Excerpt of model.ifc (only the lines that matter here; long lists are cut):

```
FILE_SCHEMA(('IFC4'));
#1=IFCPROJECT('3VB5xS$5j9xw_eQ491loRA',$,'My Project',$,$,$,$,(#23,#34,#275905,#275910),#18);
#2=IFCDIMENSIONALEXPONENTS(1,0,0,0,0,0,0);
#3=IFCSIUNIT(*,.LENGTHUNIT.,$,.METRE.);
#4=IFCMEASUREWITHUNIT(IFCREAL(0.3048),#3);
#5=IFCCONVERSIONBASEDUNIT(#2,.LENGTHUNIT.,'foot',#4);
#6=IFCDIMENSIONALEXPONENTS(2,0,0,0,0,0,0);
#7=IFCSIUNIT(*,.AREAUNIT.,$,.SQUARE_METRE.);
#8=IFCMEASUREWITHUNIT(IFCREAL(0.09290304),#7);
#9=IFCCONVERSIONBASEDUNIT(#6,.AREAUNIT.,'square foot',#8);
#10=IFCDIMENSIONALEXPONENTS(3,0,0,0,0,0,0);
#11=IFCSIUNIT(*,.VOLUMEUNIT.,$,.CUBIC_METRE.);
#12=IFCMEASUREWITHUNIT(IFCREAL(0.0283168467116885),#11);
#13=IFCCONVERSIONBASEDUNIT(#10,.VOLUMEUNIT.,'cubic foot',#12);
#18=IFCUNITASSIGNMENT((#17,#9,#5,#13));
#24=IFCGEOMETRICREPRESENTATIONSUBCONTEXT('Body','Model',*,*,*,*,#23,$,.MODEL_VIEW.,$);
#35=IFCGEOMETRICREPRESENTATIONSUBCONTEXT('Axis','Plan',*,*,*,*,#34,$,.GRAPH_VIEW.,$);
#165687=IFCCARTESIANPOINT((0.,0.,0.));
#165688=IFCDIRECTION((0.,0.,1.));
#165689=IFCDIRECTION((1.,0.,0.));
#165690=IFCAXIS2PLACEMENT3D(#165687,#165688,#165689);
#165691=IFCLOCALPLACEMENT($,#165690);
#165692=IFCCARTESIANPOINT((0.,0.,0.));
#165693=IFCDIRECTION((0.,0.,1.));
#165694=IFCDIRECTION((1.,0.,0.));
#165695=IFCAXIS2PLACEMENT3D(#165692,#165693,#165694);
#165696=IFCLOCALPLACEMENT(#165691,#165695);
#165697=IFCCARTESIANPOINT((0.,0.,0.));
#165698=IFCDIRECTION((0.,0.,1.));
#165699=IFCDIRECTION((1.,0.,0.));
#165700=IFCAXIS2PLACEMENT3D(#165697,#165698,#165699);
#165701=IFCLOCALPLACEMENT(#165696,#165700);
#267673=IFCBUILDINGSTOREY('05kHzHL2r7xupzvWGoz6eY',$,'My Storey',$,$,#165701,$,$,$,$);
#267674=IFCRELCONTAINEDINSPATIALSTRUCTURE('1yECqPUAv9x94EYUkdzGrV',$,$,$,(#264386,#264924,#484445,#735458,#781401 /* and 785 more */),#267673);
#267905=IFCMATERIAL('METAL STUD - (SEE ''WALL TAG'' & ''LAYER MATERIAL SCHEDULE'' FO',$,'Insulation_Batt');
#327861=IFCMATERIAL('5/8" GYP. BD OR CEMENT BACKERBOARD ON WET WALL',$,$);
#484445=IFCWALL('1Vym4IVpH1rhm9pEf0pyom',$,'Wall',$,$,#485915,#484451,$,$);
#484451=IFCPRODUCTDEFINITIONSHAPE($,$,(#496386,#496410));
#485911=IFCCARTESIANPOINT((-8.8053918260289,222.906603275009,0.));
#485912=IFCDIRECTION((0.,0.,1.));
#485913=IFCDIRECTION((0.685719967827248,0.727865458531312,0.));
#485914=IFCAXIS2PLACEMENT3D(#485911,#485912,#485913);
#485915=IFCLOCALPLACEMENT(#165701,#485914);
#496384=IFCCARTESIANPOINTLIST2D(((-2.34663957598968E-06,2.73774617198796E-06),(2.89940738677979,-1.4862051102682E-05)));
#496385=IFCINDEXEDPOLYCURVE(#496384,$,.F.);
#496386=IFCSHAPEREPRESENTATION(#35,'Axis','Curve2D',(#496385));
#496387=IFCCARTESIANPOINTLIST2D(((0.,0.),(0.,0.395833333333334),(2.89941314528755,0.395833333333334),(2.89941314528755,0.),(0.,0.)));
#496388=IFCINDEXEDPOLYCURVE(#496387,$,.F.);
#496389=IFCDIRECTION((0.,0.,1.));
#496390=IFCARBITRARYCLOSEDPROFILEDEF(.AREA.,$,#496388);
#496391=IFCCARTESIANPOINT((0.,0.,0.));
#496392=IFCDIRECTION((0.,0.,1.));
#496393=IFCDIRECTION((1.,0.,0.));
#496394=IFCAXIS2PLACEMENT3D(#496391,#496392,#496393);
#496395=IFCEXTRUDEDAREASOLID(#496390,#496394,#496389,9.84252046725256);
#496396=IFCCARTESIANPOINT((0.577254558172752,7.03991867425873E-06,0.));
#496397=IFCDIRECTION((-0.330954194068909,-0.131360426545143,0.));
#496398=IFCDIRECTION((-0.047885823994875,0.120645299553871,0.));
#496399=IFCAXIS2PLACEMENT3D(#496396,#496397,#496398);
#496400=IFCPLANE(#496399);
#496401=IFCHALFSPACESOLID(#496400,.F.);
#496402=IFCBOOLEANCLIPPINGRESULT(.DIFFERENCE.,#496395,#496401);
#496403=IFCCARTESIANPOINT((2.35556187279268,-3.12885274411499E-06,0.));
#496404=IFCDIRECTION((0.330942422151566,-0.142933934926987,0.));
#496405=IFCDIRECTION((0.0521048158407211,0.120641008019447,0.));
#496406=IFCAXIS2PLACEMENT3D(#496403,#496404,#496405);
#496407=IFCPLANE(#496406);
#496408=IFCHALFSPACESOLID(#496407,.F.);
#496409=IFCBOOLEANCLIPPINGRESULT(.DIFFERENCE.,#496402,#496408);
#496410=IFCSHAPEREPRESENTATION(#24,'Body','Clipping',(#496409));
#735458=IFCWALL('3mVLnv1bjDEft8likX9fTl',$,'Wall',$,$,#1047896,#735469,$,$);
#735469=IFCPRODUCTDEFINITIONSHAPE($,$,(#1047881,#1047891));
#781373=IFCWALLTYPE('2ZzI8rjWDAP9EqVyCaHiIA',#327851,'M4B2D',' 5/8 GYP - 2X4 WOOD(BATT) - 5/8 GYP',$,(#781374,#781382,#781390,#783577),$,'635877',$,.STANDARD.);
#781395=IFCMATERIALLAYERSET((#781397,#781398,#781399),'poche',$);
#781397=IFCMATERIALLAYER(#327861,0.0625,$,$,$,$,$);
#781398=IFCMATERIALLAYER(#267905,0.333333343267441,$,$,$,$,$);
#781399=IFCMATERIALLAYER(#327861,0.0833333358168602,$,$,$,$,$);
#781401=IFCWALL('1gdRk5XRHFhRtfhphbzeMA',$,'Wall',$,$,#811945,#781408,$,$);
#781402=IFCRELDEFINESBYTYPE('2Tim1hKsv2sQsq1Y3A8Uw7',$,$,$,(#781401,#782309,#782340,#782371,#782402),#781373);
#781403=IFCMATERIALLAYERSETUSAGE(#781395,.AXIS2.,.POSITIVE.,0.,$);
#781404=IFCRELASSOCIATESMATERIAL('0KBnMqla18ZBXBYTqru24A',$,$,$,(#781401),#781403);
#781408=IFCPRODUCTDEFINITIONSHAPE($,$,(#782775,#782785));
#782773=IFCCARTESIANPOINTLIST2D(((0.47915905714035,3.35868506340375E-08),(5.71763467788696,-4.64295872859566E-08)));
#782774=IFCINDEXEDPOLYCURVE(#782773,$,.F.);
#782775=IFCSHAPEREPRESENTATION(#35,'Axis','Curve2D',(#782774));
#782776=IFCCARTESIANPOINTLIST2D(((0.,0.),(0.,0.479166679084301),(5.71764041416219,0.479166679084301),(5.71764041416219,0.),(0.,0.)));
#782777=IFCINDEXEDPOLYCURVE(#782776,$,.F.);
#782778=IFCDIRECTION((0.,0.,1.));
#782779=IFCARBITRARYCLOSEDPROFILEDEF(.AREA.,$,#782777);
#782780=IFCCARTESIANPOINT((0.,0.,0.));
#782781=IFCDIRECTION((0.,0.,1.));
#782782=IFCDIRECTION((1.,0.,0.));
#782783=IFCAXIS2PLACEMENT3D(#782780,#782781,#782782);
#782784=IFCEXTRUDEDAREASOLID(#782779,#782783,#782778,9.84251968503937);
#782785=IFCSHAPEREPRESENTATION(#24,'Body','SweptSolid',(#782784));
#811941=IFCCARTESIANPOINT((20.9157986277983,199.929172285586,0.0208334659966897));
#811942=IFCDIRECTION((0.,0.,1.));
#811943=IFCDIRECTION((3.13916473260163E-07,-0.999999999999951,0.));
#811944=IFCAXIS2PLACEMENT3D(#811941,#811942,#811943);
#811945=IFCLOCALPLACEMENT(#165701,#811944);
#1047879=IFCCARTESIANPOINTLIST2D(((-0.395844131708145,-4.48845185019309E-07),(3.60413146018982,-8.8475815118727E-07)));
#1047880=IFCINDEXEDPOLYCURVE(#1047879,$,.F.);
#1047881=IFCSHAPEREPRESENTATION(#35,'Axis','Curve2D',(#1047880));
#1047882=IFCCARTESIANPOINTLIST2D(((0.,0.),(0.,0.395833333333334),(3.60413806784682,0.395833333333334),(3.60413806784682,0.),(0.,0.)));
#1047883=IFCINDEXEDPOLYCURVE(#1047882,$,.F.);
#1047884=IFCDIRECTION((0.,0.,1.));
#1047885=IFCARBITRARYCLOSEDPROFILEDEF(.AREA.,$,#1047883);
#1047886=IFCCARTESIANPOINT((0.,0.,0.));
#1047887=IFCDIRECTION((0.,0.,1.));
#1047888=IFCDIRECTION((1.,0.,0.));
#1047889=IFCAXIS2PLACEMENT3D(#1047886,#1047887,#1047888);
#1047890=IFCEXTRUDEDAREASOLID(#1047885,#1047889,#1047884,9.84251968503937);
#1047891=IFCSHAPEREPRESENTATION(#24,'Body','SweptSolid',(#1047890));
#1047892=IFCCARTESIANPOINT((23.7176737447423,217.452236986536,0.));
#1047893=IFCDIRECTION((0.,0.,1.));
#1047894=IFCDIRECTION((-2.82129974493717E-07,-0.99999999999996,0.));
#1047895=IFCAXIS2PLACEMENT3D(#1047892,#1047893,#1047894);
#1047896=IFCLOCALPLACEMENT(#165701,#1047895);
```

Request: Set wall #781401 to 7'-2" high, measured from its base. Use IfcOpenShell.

```python
import ifcopenshell
import ifcopenshell.geom
import ifcopenshell.util.representation
import ifcopenshell.util.shape
import ifcopenshell.util.unit

model = ifcopenshell.open("model.ifc")
unit_scale = ifcopenshell.util.unit.calculate_unit_scale(model)
settings = ifcopenshell.geom.settings()


def volume(element):
    """Net volume in cubic metres, openings subtracted."""
    shape = ifcopenshell.geom.create_shape(settings, element)
    return ifcopenshell.util.shape.get_volume(shape.geometry)


wall = model.by_guid("1gdRk5XRHFhRtfhphbzeMA")
before = volume(wall)

body = ifcopenshell.util.representation.get_representation(wall, "Model", "Body")
solid = body.Items[0]
old_height = solid.Depth
solid.Depth = 86 * 0.0254 / unit_scale
after = volume(wall)

print(f"height {old_height:g} -> {solid.Depth:g}, volume {before:.3f} -> {after:.3f} m3")

model.write("model_rev.ifc")
```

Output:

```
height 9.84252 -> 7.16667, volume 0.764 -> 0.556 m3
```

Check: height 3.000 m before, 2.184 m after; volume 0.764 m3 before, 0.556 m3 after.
